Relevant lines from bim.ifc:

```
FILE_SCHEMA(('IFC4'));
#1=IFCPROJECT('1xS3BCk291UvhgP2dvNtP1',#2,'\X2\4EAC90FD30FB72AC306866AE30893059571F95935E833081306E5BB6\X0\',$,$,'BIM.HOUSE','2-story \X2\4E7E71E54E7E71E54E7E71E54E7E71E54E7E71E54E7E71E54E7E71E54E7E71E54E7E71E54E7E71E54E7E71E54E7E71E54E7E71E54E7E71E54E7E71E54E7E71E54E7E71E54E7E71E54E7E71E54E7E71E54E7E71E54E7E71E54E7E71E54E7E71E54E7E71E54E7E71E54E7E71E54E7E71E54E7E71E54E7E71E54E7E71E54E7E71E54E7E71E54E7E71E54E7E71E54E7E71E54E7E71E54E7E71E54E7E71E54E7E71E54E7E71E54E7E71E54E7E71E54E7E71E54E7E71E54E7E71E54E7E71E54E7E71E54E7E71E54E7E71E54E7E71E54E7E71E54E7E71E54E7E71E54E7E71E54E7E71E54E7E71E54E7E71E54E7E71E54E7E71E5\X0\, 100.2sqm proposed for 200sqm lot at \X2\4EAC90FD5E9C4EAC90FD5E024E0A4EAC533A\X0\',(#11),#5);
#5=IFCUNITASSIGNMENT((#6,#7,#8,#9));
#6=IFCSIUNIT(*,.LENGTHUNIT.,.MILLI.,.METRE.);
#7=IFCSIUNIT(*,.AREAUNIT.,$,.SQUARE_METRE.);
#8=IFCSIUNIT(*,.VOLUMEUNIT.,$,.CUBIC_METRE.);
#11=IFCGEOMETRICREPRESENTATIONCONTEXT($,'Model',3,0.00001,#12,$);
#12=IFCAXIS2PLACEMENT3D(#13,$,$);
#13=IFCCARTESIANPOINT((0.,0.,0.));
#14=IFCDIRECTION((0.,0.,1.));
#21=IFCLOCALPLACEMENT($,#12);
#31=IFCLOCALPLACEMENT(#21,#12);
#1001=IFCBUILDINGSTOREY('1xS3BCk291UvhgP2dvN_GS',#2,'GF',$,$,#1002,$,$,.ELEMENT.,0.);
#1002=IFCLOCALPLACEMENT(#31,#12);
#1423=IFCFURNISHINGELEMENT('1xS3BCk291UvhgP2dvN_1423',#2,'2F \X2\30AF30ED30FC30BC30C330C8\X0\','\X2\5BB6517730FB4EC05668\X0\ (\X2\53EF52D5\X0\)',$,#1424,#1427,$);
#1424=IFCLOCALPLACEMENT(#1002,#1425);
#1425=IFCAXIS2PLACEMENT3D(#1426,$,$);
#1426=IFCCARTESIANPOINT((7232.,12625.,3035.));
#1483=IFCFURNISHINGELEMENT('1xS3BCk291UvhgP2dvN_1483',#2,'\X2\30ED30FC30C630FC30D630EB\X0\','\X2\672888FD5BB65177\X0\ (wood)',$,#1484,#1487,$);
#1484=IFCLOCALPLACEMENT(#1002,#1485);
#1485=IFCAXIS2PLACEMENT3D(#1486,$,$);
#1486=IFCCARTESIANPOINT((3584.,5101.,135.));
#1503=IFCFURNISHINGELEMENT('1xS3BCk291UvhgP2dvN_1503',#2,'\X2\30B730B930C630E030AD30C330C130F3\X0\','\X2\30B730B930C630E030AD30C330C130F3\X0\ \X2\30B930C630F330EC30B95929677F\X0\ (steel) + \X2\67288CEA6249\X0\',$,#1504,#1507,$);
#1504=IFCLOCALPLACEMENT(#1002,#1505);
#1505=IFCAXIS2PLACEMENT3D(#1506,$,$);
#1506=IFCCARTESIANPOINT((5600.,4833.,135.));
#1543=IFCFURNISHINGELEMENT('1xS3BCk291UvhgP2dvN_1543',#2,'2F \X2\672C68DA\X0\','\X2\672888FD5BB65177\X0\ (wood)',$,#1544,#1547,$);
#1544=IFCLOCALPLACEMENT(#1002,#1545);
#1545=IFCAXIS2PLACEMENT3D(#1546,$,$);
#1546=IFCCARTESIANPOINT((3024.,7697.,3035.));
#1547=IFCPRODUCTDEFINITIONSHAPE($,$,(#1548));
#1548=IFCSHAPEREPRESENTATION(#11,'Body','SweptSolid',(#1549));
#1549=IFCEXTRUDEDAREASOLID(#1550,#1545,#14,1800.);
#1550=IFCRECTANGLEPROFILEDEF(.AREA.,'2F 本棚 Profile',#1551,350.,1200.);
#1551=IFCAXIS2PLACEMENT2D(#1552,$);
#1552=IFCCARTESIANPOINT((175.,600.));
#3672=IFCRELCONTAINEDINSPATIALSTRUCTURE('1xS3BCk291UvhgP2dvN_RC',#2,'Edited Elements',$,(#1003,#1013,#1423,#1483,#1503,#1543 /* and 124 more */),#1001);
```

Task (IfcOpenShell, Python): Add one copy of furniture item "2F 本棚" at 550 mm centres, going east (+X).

```python
import numpy as np
import ifcopenshell
import ifcopenshell.api.geometry
import ifcopenshell.api.root
import ifcopenshell.util.element
import ifcopenshell.util.placement
import ifcopenshell.util.unit

model = ifcopenshell.open("bim.ifc")
unit_scale = ifcopenshell.util.unit.calculate_unit_scale(model)


def reuse_history(source, copy):
    """copy_class also copies each property set's owner history, people and application; keep the originals."""
    for rel in copy.IsDefinedBy:
        if rel.is_a("IfcRelDefinesByProperties") and (history := rel.RelatingPropertyDefinition.OwnerHistory):
            rel.RelatingPropertyDefinition.OwnerHistory = source.OwnerHistory
            ifcopenshell.util.element.remove_deep2(model, history)


source = model.by_guid("1xS3BCk291UvhgP2dvN_1543")
base = ifcopenshell.util.placement.get_local_placement(source.ObjectPlacement)
step = np.array([1.0, 0.0, 0.0]) * 0.55 / unit_scale

for i in range(1, 2):
    copy = ifcopenshell.api.root.copy_class(model, product=source)
    copy.Representation = ifcopenshell.util.element.copy_deep(
        model, source.Representation, exclude=["IfcGeometricRepresentationContext", "IfcRepresentationMap"]
    )
    reuse_history(source, copy)
    matrix = base.copy()
    matrix[:3, 3] += i * step
    print("added at", matrix[:3, 3].round(3) + 0.0)
    ifcopenshell.api.geometry.edit_object_placement(model, product=copy, matrix=matrix, is_si=False)

model.write("bim_updated.ifc")
```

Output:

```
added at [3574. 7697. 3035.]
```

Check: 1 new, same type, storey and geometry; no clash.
